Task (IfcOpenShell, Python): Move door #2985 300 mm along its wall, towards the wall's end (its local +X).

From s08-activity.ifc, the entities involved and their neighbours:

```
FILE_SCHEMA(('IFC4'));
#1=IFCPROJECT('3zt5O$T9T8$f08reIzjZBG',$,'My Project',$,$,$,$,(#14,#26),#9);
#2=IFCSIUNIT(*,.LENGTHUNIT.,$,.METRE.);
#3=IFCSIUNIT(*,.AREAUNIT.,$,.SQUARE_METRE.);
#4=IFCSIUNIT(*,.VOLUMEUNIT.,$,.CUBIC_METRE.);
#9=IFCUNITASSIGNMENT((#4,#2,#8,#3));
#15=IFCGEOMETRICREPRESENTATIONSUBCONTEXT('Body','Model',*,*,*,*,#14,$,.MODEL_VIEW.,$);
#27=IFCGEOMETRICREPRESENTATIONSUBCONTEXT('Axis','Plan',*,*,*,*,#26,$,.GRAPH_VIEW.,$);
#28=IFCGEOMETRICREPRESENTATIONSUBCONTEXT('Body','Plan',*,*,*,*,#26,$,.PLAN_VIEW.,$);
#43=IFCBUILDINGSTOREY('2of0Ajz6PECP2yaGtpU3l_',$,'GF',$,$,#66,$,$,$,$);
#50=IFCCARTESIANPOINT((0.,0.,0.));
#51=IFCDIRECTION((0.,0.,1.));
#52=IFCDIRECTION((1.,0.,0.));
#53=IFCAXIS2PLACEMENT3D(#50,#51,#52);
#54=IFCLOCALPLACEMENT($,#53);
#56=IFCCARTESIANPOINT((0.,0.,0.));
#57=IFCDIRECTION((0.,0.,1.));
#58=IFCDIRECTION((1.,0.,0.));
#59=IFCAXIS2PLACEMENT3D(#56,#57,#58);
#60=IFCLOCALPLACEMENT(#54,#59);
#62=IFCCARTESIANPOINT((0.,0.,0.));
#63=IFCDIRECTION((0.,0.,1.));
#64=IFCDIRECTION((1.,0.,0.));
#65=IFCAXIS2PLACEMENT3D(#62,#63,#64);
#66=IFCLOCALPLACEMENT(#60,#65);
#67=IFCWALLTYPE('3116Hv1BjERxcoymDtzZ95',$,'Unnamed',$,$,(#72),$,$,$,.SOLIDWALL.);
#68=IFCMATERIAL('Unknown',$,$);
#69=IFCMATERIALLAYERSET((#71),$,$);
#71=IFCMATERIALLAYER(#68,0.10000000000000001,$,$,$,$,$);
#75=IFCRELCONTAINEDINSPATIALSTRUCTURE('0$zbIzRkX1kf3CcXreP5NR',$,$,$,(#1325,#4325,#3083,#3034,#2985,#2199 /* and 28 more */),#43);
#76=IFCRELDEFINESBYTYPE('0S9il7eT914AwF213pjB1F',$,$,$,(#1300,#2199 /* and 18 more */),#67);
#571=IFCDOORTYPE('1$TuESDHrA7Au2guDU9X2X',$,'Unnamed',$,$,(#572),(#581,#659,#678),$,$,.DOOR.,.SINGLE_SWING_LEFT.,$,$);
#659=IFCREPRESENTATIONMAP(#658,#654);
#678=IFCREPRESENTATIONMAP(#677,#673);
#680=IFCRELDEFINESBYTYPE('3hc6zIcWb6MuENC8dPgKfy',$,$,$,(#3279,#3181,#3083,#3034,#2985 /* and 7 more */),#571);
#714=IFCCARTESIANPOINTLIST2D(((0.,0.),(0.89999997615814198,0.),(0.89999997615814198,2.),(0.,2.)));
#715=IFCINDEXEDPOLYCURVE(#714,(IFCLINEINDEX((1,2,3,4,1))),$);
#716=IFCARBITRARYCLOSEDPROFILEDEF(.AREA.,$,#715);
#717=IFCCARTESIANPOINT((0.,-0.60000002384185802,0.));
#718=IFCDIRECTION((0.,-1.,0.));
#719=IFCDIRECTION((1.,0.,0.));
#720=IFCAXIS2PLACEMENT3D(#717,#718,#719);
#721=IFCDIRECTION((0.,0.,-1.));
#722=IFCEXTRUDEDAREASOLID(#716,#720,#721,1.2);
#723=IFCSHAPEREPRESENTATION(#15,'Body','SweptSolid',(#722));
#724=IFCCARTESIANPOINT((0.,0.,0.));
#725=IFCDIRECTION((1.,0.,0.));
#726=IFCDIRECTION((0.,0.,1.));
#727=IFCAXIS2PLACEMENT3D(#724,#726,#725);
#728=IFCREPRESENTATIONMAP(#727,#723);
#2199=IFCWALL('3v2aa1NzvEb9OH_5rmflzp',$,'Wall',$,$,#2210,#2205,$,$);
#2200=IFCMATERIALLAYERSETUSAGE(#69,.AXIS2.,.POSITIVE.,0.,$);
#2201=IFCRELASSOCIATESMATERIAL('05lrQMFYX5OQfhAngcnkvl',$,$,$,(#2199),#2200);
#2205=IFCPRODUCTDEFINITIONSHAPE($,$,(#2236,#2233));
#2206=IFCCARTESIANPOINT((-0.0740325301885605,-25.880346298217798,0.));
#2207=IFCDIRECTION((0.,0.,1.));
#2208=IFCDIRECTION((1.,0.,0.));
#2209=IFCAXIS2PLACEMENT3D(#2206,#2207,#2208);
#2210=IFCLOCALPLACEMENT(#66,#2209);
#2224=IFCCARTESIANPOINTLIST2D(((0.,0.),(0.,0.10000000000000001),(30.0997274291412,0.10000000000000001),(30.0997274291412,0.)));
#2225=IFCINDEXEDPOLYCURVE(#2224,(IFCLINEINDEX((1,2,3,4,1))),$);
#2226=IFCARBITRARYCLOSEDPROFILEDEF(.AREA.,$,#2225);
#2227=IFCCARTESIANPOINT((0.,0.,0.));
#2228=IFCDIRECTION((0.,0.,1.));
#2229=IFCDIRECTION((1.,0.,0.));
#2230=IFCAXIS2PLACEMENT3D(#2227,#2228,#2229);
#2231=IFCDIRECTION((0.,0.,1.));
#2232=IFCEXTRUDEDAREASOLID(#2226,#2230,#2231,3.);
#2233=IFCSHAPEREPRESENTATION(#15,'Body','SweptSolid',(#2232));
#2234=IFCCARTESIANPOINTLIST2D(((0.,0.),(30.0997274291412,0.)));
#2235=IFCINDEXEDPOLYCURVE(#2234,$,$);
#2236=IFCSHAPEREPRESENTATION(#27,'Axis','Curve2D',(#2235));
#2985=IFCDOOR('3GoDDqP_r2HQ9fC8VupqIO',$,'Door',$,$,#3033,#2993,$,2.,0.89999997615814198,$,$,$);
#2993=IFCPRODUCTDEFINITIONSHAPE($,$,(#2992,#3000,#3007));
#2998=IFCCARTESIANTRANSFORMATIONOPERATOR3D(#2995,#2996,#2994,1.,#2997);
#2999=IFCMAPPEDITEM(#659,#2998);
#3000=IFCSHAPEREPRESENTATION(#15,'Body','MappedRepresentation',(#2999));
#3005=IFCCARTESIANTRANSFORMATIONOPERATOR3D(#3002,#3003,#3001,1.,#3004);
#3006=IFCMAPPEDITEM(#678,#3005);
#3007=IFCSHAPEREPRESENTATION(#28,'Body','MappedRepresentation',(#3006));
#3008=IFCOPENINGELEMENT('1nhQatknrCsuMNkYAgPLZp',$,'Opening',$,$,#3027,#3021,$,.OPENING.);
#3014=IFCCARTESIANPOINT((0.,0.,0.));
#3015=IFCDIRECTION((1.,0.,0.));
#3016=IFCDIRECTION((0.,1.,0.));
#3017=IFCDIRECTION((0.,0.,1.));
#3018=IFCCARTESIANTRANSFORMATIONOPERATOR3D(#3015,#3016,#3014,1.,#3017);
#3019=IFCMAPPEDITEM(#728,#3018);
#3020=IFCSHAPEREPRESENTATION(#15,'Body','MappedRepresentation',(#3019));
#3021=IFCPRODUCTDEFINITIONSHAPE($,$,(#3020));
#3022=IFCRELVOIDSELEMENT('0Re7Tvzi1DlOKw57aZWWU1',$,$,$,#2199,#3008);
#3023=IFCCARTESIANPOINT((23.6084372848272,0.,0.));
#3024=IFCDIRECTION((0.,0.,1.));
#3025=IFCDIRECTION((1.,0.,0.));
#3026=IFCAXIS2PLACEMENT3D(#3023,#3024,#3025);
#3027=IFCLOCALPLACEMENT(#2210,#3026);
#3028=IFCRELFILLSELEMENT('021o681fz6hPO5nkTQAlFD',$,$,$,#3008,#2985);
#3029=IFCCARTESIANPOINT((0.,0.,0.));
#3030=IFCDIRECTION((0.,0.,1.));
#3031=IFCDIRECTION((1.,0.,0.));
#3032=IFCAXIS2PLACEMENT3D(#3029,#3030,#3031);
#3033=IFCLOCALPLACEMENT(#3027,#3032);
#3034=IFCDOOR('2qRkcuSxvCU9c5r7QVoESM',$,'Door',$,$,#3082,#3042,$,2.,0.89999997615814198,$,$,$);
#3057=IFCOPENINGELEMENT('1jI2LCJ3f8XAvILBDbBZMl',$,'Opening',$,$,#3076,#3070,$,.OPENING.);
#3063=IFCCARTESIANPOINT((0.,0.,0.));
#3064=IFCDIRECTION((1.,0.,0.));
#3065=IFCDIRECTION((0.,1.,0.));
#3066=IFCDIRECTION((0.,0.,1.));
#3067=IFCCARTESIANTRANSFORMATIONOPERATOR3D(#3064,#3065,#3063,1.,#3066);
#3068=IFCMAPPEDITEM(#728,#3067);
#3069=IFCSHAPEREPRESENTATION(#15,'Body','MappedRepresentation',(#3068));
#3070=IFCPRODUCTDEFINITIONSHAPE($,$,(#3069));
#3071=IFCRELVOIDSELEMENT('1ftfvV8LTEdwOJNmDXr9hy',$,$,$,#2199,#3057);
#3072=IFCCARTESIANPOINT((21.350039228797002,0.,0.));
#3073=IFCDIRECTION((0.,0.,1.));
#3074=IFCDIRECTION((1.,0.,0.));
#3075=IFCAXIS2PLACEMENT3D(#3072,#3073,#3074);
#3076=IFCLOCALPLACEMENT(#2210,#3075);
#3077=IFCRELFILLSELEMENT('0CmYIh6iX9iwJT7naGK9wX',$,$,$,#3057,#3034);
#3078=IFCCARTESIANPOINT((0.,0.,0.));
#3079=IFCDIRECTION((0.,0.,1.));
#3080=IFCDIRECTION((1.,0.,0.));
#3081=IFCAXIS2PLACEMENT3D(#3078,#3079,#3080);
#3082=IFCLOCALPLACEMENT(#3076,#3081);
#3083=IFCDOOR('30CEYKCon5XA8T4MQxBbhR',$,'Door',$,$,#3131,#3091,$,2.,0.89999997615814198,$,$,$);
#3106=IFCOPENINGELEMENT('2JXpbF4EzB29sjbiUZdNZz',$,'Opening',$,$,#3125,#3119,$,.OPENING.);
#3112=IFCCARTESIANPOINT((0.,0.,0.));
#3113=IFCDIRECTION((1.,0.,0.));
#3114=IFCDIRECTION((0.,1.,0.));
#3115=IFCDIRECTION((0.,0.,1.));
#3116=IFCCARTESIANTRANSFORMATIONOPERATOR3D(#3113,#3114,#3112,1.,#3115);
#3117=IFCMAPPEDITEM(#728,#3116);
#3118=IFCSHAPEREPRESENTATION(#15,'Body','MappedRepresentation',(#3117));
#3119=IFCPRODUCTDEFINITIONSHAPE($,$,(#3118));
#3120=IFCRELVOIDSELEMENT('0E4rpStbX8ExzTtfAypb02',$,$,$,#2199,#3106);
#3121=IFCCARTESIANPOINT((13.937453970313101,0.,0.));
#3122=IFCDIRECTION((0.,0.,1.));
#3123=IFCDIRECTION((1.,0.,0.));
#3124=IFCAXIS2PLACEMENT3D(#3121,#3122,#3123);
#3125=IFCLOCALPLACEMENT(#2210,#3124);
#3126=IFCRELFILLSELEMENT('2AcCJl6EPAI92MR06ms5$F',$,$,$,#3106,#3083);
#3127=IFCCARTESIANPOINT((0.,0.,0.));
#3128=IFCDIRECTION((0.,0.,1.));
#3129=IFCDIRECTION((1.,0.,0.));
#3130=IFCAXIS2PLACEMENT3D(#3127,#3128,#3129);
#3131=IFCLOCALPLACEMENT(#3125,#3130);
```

```python
import ifcopenshell
import ifcopenshell.api.geometry
import ifcopenshell.util.placement

model = ifcopenshell.open("s08-activity.ifc")

door = model.by_guid("3GoDDqP_r2HQ9fC8VupqIO")
opening = door.FillsVoids[0].RelatingOpeningElement
wall = opening.VoidsElements[0].RelatingBuildingElement

wall_matrix = ifcopenshell.util.placement.get_local_placement(wall.ObjectPlacement)
shift = wall_matrix[:3, 0] * 0.3
before = ifcopenshell.util.placement.get_local_placement(door.ObjectPlacement)[:3, 3].copy()

# The door is placed relative to its opening, so it follows when the opening moves.
matrix = ifcopenshell.util.placement.get_local_placement(opening.ObjectPlacement)
matrix[:3, 3] += shift
ifcopenshell.api.geometry.edit_object_placement(
    model, product=opening, matrix=matrix, is_si=False, should_transform_children=True
)

after = ifcopenshell.util.placement.get_local_placement(door.ObjectPlacement)[:3, 3]
print("door moved by", (after - before).round(3) + 0.0)

model.write("s08-activity_rev.ifc")
```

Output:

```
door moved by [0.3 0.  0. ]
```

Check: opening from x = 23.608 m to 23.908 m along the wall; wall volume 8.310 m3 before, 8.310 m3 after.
